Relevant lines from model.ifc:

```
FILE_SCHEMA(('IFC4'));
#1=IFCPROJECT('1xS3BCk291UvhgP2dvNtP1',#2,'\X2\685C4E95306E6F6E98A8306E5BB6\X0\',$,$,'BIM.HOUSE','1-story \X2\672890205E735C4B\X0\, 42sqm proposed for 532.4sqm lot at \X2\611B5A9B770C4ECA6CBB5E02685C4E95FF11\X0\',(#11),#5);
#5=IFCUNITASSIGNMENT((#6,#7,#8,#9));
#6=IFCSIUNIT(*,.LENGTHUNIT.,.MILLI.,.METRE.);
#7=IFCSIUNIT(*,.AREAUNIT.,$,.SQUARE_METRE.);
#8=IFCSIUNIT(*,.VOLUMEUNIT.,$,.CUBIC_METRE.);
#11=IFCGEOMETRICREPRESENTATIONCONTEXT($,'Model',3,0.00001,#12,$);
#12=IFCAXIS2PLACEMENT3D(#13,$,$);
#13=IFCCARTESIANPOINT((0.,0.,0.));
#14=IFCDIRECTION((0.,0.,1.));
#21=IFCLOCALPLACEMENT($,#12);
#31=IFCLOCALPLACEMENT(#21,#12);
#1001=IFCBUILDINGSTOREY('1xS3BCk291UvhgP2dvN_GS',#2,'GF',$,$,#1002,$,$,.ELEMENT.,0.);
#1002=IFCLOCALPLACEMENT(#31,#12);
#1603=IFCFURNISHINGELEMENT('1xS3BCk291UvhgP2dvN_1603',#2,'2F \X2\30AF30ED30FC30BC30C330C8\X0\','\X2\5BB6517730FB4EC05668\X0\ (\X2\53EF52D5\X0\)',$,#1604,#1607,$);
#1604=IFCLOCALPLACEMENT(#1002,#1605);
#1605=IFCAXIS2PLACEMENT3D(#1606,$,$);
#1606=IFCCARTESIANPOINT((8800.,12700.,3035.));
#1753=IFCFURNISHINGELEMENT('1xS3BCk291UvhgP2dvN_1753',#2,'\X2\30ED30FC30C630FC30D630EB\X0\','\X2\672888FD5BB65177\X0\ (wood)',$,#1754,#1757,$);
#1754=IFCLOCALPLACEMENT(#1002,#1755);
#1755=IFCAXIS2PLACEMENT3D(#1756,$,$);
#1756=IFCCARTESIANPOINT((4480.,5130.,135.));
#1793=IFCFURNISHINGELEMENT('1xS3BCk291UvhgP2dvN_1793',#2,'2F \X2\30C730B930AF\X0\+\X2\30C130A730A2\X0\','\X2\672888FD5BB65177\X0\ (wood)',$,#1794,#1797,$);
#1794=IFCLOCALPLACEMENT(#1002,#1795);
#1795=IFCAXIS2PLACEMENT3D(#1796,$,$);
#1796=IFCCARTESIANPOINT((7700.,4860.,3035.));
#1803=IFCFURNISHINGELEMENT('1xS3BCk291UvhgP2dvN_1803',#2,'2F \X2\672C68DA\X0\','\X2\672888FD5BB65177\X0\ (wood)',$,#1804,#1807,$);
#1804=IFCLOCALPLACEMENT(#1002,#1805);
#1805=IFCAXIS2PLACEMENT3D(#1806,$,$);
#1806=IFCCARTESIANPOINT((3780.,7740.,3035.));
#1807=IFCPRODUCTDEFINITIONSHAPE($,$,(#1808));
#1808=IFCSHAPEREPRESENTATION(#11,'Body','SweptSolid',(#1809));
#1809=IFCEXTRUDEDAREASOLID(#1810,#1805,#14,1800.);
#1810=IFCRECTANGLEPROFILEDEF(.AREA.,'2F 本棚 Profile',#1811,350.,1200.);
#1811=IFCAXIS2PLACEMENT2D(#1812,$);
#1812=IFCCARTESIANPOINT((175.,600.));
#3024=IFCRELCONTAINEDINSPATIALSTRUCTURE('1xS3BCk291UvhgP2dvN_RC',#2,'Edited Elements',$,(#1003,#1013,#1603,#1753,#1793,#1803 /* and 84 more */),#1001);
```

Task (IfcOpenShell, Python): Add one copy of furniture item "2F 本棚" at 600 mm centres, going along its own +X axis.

```python
import ifcopenshell
import ifcopenshell.api.geometry
import ifcopenshell.api.root
import ifcopenshell.util.element
import ifcopenshell.util.placement
import ifcopenshell.util.unit

model = ifcopenshell.open("model.ifc")
unit_scale = ifcopenshell.util.unit.calculate_unit_scale(model)


def reuse_history(source, copy):
    """copy_class also copies each property set's owner history, people and application; keep the originals."""
    for rel in copy.IsDefinedBy:
        if rel.is_a("IfcRelDefinesByProperties") and (history := rel.RelatingPropertyDefinition.OwnerHistory):
            rel.RelatingPropertyDefinition.OwnerHistory = source.OwnerHistory
            ifcopenshell.util.element.remove_deep2(model, history)


source = model.by_guid("1xS3BCk291UvhgP2dvN_1803")
base = ifcopenshell.util.placement.get_local_placement(source.ObjectPlacement)
step = base[:3, 0] * 0.6 / unit_scale

for i in range(1, 2):
    copy = ifcopenshell.api.root.copy_class(model, product=source)
    copy.Representation = ifcopenshell.util.element.copy_deep(
        model, source.Representation, exclude=["IfcGeometricRepresentationContext", "IfcRepresentationMap"]
    )
    reuse_history(source, copy)
    matrix = base.copy()
    matrix[:3, 3] += i * step
    print("added at", matrix[:3, 3].round(3) + 0.0)
    ifcopenshell.api.geometry.edit_object_placement(model, product=copy, matrix=matrix, is_si=False)

model.write("model_rev.ifc")
```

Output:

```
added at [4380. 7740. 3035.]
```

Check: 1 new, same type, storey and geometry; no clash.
